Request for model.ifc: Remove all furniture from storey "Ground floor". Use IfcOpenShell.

First a look at what the model holds.

```python
import ifcopenshell
import ifcopenshell.util.element

model = ifcopenshell.open("model.ifc")
print(model.schema)
storey = next(s for s in model.by_type("IfcBuildingStorey") if s.Name == "Ground floor")
furniture = [e for e in ifcopenshell.util.element.get_decomposition(storey) if e.is_a("IfcFurnishingElement")]
seen = {}
for e in furniture:
    element_type = ifcopenshell.util.element.get_type(e)
    name = element_type.Name if element_type not in (None, e) else None
    seen[name] = seen.get(name, 0) + 1
for name, count in sorted(seen.items(), key=str):
    print(count, "x", name)
```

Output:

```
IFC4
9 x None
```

```python
import ifcopenshell
import ifcopenshell.api.root
import ifcopenshell.util.element

model = ifcopenshell.open("model.ifc")

storey = next(s for s in model.by_type("IfcBuildingStorey") if s.Name == "Ground floor")
furniture = [e for e in ifcopenshell.util.element.get_decomposition(storey) if e.is_a("IfcFurnishingElement")]

for e in furniture:
    ifcopenshell.api.root.remove_product(model, product=e)
print(len(furniture), "removed")

model.write("model-out.ifc")
```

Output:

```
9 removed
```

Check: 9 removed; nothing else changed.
